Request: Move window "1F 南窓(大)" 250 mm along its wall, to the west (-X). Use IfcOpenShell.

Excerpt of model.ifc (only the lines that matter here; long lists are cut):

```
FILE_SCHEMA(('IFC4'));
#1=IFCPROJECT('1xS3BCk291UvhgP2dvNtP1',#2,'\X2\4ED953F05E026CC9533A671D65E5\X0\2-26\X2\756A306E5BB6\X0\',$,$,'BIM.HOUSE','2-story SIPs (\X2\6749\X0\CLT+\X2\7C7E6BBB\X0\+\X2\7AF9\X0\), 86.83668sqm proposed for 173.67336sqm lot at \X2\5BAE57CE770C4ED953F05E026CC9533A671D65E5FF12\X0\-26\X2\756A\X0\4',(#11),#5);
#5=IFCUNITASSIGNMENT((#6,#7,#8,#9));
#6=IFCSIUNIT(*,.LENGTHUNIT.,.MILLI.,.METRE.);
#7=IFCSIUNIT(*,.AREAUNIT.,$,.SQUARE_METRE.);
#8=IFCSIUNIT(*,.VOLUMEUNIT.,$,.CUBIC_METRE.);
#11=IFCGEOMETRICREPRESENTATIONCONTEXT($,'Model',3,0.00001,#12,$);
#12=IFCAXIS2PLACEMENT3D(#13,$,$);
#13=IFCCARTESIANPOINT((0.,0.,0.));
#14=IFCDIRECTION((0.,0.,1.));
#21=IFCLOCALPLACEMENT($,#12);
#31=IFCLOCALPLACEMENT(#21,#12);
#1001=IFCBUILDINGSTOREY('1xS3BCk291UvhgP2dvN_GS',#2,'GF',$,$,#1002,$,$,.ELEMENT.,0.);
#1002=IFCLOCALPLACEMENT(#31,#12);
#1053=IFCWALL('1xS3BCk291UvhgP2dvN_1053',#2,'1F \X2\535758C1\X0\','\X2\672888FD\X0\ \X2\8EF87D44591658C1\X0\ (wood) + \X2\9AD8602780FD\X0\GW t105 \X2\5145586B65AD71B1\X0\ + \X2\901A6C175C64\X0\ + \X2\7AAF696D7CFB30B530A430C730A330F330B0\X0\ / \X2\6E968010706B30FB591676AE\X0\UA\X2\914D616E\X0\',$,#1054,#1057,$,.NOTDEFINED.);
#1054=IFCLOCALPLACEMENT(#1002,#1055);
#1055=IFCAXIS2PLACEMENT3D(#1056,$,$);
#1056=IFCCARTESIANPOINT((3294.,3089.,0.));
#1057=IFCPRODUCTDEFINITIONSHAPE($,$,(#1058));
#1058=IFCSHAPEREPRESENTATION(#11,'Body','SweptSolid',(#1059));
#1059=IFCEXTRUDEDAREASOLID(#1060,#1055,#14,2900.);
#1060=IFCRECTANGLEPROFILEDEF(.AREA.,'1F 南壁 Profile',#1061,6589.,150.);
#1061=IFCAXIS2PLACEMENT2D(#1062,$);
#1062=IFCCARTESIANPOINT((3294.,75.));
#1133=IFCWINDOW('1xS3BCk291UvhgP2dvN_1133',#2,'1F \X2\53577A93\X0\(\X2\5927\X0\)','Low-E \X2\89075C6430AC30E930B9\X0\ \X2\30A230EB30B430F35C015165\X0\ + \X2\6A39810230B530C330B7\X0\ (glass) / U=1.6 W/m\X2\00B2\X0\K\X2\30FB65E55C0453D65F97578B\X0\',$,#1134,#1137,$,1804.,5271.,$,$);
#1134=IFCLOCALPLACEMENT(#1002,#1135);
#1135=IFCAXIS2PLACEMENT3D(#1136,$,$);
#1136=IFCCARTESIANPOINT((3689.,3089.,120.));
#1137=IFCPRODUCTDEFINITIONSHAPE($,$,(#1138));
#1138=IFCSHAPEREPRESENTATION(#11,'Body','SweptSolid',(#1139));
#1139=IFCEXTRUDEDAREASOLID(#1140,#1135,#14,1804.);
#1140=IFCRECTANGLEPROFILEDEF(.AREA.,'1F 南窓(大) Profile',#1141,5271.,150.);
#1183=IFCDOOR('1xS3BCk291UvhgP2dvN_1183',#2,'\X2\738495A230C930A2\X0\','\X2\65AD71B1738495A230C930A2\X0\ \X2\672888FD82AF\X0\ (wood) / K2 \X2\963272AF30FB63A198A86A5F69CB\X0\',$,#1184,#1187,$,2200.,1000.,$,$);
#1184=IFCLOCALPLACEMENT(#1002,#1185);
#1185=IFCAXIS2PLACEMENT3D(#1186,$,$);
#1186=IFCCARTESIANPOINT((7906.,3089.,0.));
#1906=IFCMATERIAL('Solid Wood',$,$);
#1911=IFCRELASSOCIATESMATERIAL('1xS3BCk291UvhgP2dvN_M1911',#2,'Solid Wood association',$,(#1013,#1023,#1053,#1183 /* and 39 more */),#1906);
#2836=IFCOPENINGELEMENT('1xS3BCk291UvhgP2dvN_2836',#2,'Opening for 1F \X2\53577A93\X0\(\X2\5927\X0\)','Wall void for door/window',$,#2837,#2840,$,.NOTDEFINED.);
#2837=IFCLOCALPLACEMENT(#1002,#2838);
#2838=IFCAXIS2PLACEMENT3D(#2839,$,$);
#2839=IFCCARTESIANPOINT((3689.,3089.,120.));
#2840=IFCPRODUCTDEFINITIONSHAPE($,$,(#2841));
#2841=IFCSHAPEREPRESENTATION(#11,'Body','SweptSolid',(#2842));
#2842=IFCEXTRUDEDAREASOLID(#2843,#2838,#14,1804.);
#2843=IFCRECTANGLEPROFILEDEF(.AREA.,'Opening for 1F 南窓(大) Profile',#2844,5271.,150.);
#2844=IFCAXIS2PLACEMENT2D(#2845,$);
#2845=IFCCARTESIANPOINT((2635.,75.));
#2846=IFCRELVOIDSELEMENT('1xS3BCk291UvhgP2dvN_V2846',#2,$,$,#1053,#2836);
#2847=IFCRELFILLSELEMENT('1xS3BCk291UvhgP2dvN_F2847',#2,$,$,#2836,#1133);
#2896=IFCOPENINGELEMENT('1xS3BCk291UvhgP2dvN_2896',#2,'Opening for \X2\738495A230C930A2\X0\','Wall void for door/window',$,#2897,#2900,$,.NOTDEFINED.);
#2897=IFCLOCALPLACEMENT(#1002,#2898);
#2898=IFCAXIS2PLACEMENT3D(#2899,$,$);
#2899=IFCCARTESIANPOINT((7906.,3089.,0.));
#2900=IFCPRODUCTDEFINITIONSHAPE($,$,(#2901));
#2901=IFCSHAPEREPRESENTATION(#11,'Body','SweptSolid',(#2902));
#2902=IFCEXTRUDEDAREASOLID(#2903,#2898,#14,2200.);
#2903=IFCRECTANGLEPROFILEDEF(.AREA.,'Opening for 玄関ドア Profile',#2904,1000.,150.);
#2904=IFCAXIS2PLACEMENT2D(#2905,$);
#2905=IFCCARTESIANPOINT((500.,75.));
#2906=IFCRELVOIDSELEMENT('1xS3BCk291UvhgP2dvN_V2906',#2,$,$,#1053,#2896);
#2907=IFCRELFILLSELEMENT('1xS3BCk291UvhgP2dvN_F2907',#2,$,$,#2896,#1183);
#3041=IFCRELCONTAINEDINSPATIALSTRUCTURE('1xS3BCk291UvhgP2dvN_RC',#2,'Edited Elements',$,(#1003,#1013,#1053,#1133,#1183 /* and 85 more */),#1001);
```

```python
import ifcopenshell
import ifcopenshell.api.geometry
import ifcopenshell.util.placement

model = ifcopenshell.open("model.ifc")

window = model.by_guid("1xS3BCk291UvhgP2dvN_1133")
opening = window.FillsVoids[0].RelatingOpeningElement
wall = opening.VoidsElements[0].RelatingBuildingElement

wall_matrix = ifcopenshell.util.placement.get_local_placement(wall.ObjectPlacement)
shift = wall_matrix[:3, 0] * -250.0
before = ifcopenshell.util.placement.get_local_placement(window.ObjectPlacement)[:3, 3].copy()

# The window is not placed relative to its opening, so move both.
for product in (opening, window):
    matrix = ifcopenshell.util.placement.get_local_placement(product.ObjectPlacement)
    matrix[:3, 3] += shift
    ifcopenshell.api.geometry.edit_object_placement(model, product=product, matrix=matrix, is_si=False)

after = ifcopenshell.util.placement.get_local_placement(window.ObjectPlacement)[:3, 3]
print("window moved by", (after - before).round(3) + 0.0)

model.write("model_updated.ifc")
```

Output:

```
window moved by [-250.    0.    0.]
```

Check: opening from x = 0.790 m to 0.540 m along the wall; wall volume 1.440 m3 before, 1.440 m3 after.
